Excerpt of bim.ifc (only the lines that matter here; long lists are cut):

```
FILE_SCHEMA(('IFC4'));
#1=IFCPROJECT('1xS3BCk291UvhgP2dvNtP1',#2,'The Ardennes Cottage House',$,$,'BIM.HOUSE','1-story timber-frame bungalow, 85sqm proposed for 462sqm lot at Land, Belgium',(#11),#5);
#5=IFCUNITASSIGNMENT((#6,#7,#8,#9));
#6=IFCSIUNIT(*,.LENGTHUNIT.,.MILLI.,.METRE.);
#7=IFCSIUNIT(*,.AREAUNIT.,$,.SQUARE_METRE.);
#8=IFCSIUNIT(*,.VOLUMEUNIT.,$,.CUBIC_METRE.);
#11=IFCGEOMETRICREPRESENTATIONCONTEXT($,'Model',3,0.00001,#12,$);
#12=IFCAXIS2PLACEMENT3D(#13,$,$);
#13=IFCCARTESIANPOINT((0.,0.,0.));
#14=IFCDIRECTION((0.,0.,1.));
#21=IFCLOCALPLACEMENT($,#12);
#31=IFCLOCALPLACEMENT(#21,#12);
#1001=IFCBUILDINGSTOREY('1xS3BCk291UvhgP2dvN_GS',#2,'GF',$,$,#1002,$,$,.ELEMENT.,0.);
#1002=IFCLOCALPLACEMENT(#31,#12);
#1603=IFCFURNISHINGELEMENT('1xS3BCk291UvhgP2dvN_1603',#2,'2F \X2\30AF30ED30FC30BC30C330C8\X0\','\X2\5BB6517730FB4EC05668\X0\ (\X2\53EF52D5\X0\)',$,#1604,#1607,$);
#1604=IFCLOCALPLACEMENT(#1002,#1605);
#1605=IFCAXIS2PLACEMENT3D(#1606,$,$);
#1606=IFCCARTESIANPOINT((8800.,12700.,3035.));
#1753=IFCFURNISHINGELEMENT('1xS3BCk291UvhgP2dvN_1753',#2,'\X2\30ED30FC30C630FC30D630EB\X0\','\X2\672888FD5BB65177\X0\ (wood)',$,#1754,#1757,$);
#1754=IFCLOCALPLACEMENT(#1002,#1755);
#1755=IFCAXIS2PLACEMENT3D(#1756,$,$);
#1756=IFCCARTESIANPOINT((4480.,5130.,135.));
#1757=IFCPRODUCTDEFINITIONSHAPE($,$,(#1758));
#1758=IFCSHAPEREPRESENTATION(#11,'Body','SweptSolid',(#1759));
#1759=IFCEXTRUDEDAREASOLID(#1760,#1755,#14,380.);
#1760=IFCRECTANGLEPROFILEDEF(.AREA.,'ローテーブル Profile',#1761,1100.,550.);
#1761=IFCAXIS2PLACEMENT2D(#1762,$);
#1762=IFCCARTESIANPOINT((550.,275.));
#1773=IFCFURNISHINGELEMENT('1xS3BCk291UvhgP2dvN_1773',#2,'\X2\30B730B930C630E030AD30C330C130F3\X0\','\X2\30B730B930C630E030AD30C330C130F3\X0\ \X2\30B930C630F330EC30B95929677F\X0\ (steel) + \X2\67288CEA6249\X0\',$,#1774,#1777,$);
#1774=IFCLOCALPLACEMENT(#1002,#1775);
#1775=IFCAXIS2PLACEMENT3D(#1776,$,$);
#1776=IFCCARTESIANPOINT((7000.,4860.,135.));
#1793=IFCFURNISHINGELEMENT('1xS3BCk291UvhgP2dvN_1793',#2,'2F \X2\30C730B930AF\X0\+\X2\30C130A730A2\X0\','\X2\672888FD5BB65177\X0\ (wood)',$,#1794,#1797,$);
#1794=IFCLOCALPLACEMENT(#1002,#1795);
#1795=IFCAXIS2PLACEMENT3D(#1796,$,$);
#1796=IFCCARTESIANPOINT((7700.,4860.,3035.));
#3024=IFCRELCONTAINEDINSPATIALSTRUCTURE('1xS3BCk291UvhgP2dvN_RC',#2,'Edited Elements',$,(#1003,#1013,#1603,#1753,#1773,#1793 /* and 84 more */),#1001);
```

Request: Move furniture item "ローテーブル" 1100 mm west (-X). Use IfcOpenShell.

```python
import ifcopenshell
import ifcopenshell.api.geometry
import ifcopenshell.util.placement
import ifcopenshell.util.unit

model = ifcopenshell.open("bim.ifc")
unit_scale = ifcopenshell.util.unit.calculate_unit_scale(model)

item = model.by_guid("1xS3BCk291UvhgP2dvN_1753")
matrix = ifcopenshell.util.placement.get_local_placement(item.ObjectPlacement)
matrix[0, 3] -= 1.1 / unit_scale
ifcopenshell.api.geometry.edit_object_placement(model, product=item, matrix=matrix, is_si=False)

print(ifcopenshell.util.placement.get_local_placement(item.ObjectPlacement).round(3) + 0.0)

model.write("bim_edited.ifc")
```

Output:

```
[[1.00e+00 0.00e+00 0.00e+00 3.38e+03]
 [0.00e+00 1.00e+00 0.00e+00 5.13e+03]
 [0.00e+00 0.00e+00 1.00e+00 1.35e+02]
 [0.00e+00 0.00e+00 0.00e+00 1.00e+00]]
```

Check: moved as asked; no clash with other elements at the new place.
